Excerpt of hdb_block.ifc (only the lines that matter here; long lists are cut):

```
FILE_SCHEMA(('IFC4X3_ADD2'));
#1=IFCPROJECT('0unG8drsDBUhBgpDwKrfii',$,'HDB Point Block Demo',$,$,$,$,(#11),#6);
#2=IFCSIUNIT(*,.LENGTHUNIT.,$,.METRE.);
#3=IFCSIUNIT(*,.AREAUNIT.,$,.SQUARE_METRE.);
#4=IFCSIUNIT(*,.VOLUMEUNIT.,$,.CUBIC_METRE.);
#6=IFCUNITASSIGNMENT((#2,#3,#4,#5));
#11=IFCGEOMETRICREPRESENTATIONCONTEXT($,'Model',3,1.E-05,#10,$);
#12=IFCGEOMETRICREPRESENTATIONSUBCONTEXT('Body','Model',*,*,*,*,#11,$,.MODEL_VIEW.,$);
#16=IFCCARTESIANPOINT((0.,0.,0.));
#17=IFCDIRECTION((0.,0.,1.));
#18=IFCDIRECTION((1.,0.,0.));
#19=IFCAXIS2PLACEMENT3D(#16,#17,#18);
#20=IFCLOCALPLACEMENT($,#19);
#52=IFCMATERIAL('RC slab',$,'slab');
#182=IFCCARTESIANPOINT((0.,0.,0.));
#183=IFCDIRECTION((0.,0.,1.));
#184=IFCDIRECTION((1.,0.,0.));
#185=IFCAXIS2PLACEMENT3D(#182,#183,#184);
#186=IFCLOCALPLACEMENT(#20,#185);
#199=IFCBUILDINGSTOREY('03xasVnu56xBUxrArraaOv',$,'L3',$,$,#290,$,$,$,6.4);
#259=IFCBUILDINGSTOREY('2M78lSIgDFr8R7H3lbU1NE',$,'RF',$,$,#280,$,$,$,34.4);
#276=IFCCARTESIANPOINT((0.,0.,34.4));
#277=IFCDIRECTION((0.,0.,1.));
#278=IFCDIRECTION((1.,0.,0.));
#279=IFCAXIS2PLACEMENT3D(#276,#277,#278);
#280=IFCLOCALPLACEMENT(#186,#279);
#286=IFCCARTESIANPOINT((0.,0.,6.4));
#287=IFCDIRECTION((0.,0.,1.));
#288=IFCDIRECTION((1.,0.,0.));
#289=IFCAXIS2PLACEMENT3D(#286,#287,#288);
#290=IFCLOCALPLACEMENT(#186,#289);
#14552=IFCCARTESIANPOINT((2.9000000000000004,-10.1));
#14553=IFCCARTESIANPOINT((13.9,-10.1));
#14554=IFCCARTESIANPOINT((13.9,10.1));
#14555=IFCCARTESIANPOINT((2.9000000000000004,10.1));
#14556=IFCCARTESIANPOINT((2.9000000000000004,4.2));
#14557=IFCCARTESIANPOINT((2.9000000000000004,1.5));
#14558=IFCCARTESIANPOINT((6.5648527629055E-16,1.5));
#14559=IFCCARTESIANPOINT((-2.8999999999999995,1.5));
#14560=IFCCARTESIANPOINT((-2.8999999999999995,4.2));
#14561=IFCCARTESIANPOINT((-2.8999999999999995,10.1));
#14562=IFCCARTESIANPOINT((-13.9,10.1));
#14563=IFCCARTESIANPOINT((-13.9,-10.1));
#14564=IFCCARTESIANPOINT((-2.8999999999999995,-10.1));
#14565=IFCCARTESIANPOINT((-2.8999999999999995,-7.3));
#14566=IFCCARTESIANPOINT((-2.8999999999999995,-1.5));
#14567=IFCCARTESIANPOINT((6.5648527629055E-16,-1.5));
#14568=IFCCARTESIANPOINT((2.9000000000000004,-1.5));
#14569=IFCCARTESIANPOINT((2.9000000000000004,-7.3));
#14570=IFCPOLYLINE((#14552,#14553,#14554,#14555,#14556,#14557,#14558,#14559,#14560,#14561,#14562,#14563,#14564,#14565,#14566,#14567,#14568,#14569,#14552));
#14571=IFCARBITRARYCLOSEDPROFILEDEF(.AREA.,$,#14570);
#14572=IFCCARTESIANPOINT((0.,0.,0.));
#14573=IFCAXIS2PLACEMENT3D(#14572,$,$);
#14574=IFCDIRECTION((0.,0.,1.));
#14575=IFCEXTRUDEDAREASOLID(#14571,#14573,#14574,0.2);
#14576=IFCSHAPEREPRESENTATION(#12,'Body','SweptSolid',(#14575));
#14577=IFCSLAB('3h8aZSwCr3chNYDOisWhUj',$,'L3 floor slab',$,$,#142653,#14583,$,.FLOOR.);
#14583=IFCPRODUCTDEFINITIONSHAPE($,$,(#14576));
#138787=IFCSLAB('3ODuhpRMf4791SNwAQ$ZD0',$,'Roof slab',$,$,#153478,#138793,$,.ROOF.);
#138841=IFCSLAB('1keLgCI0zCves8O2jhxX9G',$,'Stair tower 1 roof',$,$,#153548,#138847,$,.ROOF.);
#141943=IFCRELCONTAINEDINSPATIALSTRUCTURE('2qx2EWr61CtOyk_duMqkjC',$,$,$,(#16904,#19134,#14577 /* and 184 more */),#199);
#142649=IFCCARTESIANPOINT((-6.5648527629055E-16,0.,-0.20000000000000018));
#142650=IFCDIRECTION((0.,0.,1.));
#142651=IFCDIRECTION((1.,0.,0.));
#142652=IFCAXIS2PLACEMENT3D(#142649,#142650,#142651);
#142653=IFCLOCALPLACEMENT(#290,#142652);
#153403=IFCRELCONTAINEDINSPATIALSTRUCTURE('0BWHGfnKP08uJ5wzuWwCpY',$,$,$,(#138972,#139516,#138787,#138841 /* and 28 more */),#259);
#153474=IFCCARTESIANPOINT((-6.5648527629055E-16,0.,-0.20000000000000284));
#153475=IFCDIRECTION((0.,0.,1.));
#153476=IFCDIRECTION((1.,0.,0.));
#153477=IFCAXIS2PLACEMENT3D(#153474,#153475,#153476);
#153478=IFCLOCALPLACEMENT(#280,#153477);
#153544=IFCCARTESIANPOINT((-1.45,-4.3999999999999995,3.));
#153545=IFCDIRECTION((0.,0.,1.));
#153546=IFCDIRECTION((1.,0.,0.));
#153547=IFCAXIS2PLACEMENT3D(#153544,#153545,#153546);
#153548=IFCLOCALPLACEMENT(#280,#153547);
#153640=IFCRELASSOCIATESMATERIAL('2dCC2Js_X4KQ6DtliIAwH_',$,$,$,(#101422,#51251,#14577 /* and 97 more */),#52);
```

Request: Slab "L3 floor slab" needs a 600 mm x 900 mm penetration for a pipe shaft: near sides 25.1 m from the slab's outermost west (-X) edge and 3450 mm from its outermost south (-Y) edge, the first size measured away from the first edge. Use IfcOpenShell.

```python
import numpy as np
import ifcopenshell
import ifcopenshell.api.feature
import ifcopenshell.api.geometry
import ifcopenshell.api.root
import ifcopenshell.geom
import ifcopenshell.util.placement
import ifcopenshell.util.representation
import ifcopenshell.util.shape
import ifcopenshell.util.unit

model = ifcopenshell.open("hdb_block.ifc")
unit_scale = ifcopenshell.util.unit.calculate_unit_scale(model)
settings = ifcopenshell.geom.settings()


def volume(element):
    """Net volume in cubic metres, openings subtracted."""
    shape = ifcopenshell.geom.create_shape(settings, element)
    return ifcopenshell.util.shape.get_volume(shape.geometry)


slab = model.by_guid("3h8aZSwCr3chNYDOisWhUj")
before = volume(slab)

# Extent in the slab's own axes, in metres. The edges named are its -X and -Y sides.
slab_shape = ifcopenshell.geom.create_shape(settings, slab)
vertices = ifcopenshell.util.shape.get_vertices(slab_shape.geometry)
x_min, y_min, bottom = vertices.min(axis=0)
top = vertices[:, 2].max()

opening = ifcopenshell.api.root.create_entity(model, ifc_class="IfcOpeningElement", name="Pipe shaft opening", predefined_type="OPENING")
context = ifcopenshell.util.representation.get_context(model, "Model", "Body", "MODEL_VIEW")
width, depth = 0.6, 0.9
outline = [(0.0, 0.0), (width, 0.0), (width, depth), (0.0, depth), (0.0, 0.0)]
# Overshoot both faces by 50 mm so the cut is clean.
shape = ifcopenshell.api.geometry.add_slab_representation(
    model, context=context, depth=top - bottom + 0.1, polyline=outline
)
ifcopenshell.api.geometry.assign_representation(model, product=opening, representation=shape)

matrix = ifcopenshell.util.placement.get_local_placement(slab.ObjectPlacement)
matrix[:, 3] = matrix @ np.append(np.array([x_min + 25.1, y_min + 3.45, bottom - 0.05]) / unit_scale, 1.0)
ifcopenshell.api.geometry.edit_object_placement(model, product=opening, matrix=matrix, is_si=False)
ifcopenshell.api.feature.add_feature(model, feature=opening, element=slab)

after = volume(slab)

print(f"slab volume {before:.3f} -> {after:.3f} m3")

model.write("hdb_block-out.ifc")
```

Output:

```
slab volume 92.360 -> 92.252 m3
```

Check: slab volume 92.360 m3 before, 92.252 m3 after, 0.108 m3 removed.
